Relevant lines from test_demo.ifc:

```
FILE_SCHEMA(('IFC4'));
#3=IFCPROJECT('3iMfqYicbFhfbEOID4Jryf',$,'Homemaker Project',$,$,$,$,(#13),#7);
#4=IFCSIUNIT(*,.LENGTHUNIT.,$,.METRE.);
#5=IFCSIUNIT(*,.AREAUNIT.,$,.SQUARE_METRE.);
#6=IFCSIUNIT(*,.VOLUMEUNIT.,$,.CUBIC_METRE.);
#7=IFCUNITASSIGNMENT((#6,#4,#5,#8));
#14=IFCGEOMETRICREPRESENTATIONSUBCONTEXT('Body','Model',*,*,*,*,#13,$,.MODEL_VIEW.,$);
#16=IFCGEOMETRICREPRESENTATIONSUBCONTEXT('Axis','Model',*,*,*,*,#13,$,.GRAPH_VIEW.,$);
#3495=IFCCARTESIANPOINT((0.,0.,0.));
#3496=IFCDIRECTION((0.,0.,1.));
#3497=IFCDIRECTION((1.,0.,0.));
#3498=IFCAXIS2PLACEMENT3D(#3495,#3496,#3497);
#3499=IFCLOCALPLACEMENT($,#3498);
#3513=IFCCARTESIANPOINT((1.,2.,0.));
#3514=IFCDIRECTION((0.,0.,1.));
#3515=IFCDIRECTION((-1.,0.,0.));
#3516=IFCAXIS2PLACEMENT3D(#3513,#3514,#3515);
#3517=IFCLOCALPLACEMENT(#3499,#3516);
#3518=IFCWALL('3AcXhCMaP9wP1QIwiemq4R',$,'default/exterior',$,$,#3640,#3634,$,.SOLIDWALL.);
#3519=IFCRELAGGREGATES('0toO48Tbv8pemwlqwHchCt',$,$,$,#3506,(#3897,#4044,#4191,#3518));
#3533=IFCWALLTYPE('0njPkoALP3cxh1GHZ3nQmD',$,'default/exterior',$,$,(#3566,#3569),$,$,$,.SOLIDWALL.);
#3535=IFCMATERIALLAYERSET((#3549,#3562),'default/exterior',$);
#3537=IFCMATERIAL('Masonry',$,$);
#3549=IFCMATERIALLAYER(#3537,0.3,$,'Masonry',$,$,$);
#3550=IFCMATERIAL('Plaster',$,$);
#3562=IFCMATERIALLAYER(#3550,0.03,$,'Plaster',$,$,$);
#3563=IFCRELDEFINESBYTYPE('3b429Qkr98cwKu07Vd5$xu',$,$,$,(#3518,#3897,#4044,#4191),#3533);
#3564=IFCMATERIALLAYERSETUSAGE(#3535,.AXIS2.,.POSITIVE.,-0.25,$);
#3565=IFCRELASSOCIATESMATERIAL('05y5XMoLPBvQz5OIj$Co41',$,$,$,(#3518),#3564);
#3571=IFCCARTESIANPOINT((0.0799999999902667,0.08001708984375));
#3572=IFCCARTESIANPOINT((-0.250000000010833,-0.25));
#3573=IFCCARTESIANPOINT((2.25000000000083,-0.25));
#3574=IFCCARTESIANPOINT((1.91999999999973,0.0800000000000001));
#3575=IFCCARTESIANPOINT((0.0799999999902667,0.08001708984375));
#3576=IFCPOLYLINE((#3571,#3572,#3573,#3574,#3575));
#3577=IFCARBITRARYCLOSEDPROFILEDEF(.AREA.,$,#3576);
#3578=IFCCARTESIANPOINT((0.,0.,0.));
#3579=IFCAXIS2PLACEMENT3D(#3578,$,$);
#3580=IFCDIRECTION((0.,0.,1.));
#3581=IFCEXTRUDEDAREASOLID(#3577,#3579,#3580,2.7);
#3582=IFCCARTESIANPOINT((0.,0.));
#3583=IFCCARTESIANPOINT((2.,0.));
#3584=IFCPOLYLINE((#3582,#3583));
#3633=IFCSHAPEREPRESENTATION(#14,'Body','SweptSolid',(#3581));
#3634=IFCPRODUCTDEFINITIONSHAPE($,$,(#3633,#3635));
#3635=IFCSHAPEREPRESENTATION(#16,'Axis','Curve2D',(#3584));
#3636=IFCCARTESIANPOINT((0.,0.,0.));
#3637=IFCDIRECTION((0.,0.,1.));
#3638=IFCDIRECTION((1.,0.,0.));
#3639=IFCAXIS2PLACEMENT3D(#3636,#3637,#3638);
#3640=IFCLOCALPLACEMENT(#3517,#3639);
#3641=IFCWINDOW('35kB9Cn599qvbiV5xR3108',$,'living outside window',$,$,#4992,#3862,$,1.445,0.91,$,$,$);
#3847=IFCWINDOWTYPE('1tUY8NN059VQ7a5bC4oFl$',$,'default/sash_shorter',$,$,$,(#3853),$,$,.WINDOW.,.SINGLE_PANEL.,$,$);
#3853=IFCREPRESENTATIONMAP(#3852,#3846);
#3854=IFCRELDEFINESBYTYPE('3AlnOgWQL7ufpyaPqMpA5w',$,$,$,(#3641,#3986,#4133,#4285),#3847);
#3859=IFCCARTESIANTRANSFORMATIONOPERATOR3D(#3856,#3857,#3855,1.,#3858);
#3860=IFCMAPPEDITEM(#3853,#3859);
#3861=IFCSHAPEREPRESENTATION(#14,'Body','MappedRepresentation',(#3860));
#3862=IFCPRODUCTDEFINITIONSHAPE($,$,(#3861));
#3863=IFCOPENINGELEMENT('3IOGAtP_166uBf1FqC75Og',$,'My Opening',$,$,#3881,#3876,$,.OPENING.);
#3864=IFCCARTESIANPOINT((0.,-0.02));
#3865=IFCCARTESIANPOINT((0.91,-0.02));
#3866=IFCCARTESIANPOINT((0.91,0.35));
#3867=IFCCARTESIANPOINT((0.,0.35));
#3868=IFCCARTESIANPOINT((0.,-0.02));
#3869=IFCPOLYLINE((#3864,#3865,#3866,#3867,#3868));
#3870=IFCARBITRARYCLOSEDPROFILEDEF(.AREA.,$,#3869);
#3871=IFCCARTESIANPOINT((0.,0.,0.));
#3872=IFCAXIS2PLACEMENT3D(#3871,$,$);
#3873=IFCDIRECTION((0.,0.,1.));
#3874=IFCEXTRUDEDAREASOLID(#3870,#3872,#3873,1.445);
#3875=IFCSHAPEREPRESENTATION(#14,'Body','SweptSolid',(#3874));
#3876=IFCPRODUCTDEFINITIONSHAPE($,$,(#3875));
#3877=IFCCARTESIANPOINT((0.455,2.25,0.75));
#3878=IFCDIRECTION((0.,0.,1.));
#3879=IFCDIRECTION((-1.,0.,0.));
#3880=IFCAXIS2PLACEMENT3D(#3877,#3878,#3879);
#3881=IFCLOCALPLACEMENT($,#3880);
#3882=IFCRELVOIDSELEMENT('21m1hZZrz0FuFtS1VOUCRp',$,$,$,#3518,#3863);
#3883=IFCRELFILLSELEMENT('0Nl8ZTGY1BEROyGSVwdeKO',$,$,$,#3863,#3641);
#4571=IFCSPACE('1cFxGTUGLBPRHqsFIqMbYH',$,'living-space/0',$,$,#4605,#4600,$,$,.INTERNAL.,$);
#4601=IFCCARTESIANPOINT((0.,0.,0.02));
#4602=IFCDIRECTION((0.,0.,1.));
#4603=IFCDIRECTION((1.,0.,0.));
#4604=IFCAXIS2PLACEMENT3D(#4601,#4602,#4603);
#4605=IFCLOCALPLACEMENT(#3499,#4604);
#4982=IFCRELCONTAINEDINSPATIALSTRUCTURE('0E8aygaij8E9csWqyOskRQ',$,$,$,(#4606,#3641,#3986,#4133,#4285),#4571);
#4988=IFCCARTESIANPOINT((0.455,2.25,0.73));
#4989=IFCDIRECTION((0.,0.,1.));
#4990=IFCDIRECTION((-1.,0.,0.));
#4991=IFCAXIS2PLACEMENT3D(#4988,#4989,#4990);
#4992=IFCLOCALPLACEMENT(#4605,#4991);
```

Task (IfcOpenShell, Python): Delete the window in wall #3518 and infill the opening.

```python
import ifcopenshell
import ifcopenshell.api.feature
import ifcopenshell.api.root
import ifcopenshell.geom
import ifcopenshell.util.shape

model = ifcopenshell.open("test_demo.ifc")
settings = ifcopenshell.geom.settings()


def volume(element):
    """Net volume in cubic metres, openings subtracted."""
    shape = ifcopenshell.geom.create_shape(settings, element)
    return ifcopenshell.util.shape.get_volume(shape.geometry)


window = model.by_guid("35kB9Cn599qvbiV5xR3108")
opening = window.FillsVoids[0].RelatingOpeningElement
wall = opening.VoidsElements[0].RelatingBuildingElement
before = volume(wall)

ifcopenshell.api.root.remove_product(model, product=window)
ifcopenshell.api.feature.remove_feature(model, feature=opening)

after = volume(wall)

print(f"wall volume {before:.3f} -> {after:.3f} m3")

model.write("test_demo-out.ifc")
```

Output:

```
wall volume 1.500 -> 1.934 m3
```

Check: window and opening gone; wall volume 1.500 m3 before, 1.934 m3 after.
